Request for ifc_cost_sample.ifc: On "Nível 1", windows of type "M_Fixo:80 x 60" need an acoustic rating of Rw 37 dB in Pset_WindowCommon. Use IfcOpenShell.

First a look at what the model holds.

```python
import ifcopenshell
import ifcopenshell.util.element

model = ifcopenshell.open("ifc_cost_sample.ifc")
print(model.schema)
storey = next(s for s in model.by_type("IfcBuildingStorey") if s.Name == "Nível 1")
windows = [e for e in ifcopenshell.util.element.get_decomposition(storey) if e.is_a("IfcWindow")]
seen = {}
for e in windows:
    element_type = ifcopenshell.util.element.get_type(e)
    key = (element_type.Name if element_type != e and element_type else None, ifcopenshell.util.element.get_pset(e, "Pset_WindowCommon", "AcousticRating"))
    seen[key] = seen.get(key, 0) + 1
for (name, value), count in sorted(seen.items(), key=str):
    print(count, "x", name, "|", value)
```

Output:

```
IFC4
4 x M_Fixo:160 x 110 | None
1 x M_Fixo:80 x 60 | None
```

```python
import ifcopenshell
import ifcopenshell.api.pset
import ifcopenshell.util.element

model = ifcopenshell.open("ifc_cost_sample.ifc")

storey = next(s for s in model.by_type("IfcBuildingStorey") if s.Name == "Nível 1")
windows = [e for e in ifcopenshell.util.element.get_decomposition(storey) if e.is_a("IfcWindow")]

count = 0
for e in windows:
    element_type = ifcopenshell.util.element.get_type(e)
    if element_type in (None, e) or element_type.Name != "M_Fixo:80 x 60":
        continue
    # add_pset returns the element's existing set when there is one.
    pset = ifcopenshell.api.pset.add_pset(model, product=e, name="Pset_WindowCommon")
    ifcopenshell.api.pset.edit_pset(model, pset=pset, properties={"AcousticRating": "Rw 37 dB"})
    count += 1

print(count, "windows updated")

model.write("ifc_cost_sample_rev.ifc")
```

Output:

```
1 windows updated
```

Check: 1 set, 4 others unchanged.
